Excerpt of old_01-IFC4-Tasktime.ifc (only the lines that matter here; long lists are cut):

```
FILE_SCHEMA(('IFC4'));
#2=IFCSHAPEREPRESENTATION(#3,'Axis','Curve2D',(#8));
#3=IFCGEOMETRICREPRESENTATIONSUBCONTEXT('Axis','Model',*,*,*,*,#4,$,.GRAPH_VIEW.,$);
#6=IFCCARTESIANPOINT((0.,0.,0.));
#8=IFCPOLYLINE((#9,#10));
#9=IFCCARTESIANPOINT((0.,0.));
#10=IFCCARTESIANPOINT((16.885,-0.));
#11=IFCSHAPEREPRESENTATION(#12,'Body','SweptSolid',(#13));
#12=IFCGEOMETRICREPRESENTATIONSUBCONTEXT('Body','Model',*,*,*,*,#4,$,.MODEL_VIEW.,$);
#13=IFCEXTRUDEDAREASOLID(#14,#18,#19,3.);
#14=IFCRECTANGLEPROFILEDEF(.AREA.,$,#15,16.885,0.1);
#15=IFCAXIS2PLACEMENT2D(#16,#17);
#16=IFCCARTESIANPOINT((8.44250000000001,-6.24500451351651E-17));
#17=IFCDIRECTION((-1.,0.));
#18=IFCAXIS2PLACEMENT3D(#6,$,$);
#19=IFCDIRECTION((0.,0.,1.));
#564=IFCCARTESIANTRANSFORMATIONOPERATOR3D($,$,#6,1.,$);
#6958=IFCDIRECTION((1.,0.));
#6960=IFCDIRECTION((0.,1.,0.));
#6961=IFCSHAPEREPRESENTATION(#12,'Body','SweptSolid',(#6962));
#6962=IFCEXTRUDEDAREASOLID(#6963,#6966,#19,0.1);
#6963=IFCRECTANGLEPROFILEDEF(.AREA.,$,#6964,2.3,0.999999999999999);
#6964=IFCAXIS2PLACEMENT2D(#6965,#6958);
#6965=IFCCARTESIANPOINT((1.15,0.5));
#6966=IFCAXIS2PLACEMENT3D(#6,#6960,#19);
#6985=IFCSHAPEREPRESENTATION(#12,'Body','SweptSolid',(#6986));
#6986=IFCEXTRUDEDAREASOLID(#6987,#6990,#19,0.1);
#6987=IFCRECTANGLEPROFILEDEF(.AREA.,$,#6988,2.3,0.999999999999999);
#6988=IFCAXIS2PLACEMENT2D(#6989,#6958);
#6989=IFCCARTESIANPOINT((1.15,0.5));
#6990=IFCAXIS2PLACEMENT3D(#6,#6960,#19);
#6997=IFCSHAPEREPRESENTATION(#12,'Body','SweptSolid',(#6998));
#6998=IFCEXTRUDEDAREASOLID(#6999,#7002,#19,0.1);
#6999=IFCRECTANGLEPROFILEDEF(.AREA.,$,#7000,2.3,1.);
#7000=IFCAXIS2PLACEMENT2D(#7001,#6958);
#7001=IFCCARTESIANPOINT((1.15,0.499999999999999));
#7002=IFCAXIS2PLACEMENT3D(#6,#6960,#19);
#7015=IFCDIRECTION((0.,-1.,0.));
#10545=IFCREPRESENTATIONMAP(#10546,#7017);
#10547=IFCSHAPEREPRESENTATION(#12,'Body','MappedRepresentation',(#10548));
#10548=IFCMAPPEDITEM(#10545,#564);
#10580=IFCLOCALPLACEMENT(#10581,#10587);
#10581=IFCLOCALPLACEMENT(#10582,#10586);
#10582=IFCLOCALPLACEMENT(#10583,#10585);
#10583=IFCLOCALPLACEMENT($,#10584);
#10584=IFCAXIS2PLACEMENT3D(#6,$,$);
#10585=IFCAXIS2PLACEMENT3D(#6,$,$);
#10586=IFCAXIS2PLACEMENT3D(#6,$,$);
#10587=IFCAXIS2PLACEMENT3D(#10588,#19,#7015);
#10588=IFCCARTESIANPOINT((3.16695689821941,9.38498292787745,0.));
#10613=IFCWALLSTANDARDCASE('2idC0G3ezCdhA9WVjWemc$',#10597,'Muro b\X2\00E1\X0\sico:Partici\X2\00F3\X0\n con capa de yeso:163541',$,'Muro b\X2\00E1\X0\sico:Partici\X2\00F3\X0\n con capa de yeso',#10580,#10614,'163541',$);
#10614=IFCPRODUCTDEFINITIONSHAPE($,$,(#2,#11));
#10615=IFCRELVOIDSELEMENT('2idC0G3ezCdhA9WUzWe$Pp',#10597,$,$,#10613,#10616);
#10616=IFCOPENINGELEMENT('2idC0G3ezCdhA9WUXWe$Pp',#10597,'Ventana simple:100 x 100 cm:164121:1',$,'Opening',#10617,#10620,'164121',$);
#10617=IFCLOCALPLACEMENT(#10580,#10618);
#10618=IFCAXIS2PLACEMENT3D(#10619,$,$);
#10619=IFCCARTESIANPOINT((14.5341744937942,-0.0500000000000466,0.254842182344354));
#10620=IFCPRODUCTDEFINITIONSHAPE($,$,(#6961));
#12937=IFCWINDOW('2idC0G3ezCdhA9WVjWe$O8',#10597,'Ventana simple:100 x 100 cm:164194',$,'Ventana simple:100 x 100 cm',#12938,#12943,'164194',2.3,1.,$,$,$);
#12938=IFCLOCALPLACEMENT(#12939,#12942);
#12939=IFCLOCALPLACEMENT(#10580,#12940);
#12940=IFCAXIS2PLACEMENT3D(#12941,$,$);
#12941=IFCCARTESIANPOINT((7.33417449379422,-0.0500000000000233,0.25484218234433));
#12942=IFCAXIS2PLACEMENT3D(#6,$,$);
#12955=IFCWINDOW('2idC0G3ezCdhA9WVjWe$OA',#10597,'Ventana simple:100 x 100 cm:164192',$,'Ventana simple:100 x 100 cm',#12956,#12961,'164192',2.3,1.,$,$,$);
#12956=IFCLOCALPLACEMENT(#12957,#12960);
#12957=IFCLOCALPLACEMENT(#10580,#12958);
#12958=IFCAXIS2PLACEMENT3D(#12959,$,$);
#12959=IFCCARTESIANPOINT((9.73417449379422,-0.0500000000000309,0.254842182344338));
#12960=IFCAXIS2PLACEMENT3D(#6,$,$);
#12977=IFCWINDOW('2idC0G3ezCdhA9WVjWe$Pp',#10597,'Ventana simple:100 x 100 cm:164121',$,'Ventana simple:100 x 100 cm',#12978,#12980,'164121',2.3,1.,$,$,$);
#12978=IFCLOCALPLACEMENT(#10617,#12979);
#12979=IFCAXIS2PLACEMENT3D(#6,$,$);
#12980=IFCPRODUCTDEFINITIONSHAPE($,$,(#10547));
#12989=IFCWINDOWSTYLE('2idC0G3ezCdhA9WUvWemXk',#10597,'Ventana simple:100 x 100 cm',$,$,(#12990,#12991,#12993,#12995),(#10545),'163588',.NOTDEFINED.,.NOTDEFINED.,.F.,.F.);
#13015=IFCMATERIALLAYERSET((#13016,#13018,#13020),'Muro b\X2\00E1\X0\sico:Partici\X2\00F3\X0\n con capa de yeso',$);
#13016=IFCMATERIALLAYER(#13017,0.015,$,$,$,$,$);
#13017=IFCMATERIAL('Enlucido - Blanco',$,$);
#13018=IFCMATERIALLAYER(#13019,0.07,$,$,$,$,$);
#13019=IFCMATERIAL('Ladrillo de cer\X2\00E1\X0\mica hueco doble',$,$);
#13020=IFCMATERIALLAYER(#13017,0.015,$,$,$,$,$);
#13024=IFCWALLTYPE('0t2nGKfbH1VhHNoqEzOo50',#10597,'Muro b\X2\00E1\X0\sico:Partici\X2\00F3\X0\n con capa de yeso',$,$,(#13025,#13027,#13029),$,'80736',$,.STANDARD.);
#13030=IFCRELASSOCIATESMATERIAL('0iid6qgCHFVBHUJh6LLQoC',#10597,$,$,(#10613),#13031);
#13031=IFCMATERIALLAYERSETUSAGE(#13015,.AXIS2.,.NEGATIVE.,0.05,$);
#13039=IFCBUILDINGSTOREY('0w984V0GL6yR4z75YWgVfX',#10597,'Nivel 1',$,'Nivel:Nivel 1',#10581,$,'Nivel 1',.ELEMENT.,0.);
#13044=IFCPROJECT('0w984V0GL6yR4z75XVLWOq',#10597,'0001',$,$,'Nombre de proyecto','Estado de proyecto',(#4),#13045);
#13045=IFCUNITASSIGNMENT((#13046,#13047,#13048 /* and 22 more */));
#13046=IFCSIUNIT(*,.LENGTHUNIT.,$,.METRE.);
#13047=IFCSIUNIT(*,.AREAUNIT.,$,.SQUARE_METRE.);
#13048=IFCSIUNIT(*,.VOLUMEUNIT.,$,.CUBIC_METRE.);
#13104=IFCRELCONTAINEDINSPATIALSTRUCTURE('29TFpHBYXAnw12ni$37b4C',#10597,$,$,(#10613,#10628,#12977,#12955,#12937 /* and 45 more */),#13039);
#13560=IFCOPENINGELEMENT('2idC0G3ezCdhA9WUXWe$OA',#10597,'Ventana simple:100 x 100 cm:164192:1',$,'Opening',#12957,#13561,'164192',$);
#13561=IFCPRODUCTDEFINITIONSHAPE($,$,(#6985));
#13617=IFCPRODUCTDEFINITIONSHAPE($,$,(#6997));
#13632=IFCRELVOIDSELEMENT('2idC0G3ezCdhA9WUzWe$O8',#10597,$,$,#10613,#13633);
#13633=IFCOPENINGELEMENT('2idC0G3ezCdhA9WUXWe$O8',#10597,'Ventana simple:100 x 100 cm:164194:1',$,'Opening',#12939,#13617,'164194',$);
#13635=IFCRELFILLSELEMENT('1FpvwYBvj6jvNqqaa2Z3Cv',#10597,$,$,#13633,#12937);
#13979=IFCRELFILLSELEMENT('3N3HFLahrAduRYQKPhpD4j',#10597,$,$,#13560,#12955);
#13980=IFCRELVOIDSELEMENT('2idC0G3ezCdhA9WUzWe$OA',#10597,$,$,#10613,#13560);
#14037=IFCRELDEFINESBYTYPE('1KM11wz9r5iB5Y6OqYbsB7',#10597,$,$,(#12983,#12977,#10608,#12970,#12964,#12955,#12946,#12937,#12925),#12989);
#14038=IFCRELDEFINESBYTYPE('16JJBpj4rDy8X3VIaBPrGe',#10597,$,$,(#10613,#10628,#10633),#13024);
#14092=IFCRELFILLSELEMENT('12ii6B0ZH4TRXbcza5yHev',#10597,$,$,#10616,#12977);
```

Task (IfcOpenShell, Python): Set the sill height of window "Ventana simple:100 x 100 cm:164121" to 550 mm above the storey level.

```python
import numpy as np
import ifcopenshell
import ifcopenshell.api.geometry
import ifcopenshell.geom
import ifcopenshell.util.element
import ifcopenshell.util.placement
import ifcopenshell.util.shape
import ifcopenshell.util.unit

model = ifcopenshell.open("old_01-IFC4-Tasktime.ifc")
unit_scale = ifcopenshell.util.unit.calculate_unit_scale(model)

window = model.by_id(12977)
opening = window.FillsVoids[0].RelatingOpeningElement
storey = ifcopenshell.util.element.get_container(window, ifc_class="IfcBuildingStorey")
level = ifcopenshell.util.placement.get_local_placement(storey.ObjectPlacement)[2, 3]

# The opening's origin need not be at the sill, so measure its lowest point.
shape = ifcopenshell.geom.create_shape(ifcopenshell.geom.settings(), opening)
bottom = ifcopenshell.util.shape.get_shape_bottom_elevation(shape, shape.geometry) / unit_scale
dz = level + 0.55 - bottom

shift = np.array([0.0, 0.0, dz])
# The window is placed relative to its opening, so it follows when the opening moves.
matrix = ifcopenshell.util.placement.get_local_placement(opening.ObjectPlacement)
matrix[:3, 3] += shift
ifcopenshell.api.geometry.edit_object_placement(
    model, product=opening, matrix=matrix, is_si=False, should_transform_children=True
)

print(f"moved by {dz * unit_scale:+.3f} m")

model.write("old_01-IFC4-Tasktime_rev.ifc")
```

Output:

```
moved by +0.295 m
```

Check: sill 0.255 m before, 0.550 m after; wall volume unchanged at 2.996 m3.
